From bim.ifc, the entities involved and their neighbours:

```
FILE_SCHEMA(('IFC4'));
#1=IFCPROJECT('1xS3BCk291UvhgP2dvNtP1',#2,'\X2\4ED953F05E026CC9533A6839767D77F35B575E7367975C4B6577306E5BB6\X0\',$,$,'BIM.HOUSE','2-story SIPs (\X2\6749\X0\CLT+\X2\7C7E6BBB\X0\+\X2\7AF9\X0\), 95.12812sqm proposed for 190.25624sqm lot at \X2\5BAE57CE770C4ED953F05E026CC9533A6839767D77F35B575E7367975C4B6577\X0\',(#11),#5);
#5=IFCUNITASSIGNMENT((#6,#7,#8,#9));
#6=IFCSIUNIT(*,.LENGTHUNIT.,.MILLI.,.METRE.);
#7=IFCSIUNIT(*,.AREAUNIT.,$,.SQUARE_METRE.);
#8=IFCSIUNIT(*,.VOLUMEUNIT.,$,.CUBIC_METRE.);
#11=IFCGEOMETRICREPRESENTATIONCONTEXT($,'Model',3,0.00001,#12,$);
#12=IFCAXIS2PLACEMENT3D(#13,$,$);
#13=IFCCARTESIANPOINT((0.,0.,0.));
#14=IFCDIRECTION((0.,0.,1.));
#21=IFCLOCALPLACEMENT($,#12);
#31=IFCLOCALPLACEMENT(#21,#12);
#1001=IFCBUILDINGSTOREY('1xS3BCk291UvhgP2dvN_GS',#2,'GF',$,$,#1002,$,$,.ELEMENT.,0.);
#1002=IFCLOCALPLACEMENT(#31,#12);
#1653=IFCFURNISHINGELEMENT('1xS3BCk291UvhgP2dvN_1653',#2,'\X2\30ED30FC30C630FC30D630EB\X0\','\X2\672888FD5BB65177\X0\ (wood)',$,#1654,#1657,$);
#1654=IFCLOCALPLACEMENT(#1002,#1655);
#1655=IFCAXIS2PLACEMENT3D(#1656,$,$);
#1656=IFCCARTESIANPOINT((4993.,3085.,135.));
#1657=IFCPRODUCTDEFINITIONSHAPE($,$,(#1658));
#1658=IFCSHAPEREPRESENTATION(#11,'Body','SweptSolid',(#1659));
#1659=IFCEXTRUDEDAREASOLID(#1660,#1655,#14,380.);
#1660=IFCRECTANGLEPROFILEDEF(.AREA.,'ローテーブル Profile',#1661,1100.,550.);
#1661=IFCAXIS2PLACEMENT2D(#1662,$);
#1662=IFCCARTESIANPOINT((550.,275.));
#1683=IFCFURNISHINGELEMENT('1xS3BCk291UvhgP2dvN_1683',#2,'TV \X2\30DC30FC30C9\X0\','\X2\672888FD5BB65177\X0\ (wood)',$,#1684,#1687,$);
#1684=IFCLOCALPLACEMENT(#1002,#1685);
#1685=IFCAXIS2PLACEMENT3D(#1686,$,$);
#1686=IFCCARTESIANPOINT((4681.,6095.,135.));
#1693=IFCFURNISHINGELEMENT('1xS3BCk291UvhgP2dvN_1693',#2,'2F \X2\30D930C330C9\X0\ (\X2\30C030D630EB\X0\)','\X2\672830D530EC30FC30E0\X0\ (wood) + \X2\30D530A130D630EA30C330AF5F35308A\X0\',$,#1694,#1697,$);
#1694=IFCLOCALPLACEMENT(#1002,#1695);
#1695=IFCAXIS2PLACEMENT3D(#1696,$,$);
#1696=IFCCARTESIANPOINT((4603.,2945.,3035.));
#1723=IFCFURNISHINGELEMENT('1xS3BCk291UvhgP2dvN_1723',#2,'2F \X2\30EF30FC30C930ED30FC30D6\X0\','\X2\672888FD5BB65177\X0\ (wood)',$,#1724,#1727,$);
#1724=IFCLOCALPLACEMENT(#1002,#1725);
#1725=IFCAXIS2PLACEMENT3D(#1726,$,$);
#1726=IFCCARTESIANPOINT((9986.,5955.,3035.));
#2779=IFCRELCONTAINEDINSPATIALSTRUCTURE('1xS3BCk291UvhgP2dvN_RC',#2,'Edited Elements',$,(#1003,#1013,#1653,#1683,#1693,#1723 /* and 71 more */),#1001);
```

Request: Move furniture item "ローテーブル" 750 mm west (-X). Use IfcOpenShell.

```python
import ifcopenshell
import ifcopenshell.api.geometry
import ifcopenshell.util.placement
import ifcopenshell.util.unit

model = ifcopenshell.open("bim.ifc")
unit_scale = ifcopenshell.util.unit.calculate_unit_scale(model)

item = model.by_guid("1xS3BCk291UvhgP2dvN_1653")
matrix = ifcopenshell.util.placement.get_local_placement(item.ObjectPlacement)
matrix[0, 3] -= 0.75 / unit_scale
ifcopenshell.api.geometry.edit_object_placement(model, product=item, matrix=matrix, is_si=False)

print(ifcopenshell.util.placement.get_local_placement(item.ObjectPlacement).round(3) + 0.0)

model.write("bim-out.ifc")
```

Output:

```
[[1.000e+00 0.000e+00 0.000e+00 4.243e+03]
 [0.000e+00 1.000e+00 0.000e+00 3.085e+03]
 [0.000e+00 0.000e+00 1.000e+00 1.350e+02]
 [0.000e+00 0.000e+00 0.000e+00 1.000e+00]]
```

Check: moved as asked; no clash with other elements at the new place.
